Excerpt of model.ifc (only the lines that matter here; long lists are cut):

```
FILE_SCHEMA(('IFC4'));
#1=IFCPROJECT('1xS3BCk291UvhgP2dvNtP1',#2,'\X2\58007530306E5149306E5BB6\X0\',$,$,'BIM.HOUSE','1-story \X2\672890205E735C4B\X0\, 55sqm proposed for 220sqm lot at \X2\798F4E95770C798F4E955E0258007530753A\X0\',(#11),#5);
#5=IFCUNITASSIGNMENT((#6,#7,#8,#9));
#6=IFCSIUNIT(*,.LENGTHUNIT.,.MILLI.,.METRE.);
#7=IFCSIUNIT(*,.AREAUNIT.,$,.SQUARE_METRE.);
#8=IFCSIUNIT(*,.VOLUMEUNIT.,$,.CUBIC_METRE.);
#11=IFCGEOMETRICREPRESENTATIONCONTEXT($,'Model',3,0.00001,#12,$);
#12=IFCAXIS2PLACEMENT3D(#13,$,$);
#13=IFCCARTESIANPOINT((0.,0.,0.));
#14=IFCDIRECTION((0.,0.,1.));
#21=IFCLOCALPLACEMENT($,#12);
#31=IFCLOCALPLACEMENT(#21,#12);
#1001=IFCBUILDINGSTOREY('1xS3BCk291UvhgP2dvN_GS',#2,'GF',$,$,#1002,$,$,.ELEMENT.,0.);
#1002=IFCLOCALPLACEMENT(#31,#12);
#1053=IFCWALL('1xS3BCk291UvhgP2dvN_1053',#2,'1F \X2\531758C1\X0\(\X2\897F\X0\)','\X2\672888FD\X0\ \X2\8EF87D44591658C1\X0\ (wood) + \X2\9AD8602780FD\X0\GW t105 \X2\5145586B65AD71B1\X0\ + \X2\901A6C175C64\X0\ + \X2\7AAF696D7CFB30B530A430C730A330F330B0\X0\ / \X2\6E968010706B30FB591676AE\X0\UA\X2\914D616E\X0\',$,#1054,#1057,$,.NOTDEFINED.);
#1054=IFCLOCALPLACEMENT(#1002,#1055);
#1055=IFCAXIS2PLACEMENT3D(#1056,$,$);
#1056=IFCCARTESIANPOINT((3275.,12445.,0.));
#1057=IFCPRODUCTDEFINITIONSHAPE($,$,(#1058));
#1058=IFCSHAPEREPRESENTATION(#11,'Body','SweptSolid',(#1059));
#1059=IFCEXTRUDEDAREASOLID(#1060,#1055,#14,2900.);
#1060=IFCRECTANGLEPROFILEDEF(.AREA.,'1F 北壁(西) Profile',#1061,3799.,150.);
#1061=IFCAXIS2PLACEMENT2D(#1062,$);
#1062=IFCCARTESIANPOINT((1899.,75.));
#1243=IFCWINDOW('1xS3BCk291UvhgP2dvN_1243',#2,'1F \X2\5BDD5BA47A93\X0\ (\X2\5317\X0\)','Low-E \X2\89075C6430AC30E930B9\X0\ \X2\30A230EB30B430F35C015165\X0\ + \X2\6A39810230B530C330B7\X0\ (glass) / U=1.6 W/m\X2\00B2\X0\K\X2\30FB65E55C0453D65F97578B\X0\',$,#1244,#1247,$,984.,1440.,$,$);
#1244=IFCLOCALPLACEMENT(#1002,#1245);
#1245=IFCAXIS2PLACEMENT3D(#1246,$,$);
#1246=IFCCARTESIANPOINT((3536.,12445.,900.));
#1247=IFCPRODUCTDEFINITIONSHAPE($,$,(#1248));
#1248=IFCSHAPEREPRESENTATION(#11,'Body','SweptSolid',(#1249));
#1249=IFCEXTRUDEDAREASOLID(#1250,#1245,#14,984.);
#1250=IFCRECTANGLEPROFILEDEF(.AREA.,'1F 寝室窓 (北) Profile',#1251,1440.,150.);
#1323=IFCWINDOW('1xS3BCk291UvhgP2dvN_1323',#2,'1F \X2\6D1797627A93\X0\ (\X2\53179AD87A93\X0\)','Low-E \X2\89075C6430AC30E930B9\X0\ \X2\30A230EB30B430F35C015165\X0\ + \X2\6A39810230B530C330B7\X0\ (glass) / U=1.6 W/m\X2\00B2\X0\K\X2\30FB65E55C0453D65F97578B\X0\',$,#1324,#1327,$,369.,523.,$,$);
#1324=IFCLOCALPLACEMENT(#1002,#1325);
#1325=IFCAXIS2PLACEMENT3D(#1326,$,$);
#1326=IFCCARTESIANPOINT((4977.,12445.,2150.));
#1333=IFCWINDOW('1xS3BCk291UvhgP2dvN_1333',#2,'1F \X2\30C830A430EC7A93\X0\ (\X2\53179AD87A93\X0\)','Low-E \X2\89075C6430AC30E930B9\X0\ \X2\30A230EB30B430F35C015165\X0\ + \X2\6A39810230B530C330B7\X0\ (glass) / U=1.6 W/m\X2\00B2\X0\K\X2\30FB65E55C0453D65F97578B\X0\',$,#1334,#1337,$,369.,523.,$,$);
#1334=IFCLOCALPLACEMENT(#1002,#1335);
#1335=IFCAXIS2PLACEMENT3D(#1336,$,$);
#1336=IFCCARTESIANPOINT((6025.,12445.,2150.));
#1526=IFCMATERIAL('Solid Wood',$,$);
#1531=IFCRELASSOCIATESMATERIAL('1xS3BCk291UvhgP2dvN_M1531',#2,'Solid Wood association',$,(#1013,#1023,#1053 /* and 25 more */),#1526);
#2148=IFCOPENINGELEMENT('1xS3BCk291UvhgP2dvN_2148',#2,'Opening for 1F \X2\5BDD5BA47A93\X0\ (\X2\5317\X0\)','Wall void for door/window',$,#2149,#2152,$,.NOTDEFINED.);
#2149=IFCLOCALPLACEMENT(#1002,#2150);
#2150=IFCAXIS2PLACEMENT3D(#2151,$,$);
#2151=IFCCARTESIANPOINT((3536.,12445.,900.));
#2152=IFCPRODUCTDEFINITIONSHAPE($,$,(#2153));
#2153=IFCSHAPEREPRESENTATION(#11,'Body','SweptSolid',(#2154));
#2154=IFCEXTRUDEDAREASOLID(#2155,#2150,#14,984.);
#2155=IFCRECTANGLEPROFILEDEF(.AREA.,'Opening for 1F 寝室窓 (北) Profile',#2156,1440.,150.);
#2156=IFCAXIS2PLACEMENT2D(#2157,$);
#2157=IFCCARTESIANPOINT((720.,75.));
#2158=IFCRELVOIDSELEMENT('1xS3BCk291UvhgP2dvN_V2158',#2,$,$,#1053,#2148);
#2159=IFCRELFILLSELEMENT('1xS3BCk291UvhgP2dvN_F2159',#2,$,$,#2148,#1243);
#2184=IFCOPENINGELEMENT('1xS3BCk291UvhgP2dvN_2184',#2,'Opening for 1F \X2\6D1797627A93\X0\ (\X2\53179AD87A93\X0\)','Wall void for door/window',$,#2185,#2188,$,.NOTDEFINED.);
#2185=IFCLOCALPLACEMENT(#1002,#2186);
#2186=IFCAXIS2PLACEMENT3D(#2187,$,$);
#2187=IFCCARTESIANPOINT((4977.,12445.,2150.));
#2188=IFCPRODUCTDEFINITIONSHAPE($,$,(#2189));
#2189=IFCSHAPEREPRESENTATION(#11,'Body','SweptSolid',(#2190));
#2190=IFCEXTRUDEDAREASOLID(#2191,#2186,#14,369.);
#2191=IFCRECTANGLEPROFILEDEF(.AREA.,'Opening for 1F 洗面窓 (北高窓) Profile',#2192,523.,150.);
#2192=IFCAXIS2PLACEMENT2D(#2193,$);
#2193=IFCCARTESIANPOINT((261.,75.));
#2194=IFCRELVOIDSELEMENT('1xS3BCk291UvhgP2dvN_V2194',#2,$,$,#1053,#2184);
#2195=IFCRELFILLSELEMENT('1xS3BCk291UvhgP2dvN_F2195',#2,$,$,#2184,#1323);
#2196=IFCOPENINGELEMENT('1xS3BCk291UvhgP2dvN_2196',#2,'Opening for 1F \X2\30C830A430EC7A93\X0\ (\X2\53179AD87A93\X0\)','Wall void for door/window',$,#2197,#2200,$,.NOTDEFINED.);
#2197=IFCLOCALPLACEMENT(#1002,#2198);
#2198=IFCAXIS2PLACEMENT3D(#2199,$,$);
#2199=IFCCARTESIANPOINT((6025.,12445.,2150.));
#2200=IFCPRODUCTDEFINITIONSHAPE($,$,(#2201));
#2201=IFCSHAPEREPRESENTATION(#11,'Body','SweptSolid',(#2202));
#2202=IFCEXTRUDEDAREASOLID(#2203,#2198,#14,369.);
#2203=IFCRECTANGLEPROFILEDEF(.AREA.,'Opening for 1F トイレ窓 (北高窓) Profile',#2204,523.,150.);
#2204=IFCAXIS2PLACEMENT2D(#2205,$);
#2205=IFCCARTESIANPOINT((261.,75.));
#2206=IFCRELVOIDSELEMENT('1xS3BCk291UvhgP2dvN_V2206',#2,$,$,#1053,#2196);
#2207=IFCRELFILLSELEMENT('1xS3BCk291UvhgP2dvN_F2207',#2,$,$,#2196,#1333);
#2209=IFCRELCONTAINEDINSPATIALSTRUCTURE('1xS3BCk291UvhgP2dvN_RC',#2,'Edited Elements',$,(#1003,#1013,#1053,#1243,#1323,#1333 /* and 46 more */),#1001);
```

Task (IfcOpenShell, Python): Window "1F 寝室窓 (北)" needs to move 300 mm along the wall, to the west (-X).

```python
import ifcopenshell
import ifcopenshell.api.geometry
import ifcopenshell.util.placement
import ifcopenshell.util.unit

model = ifcopenshell.open("model.ifc")
unit_scale = ifcopenshell.util.unit.calculate_unit_scale(model)

window = model.by_guid("1xS3BCk291UvhgP2dvN_1243")
opening = window.FillsVoids[0].RelatingOpeningElement
wall = opening.VoidsElements[0].RelatingBuildingElement

wall_matrix = ifcopenshell.util.placement.get_local_placement(wall.ObjectPlacement)
shift = wall_matrix[:3, 0] * -0.3 / unit_scale
before = ifcopenshell.util.placement.get_local_placement(window.ObjectPlacement)[:3, 3].copy()

# The window is not placed relative to its opening, so move both.
for product in (opening, window):
    matrix = ifcopenshell.util.placement.get_local_placement(product.ObjectPlacement)
    matrix[:3, 3] += shift
    ifcopenshell.api.geometry.edit_object_placement(model, product=product, matrix=matrix, is_si=False)

after = ifcopenshell.util.placement.get_local_placement(window.ObjectPlacement)[:3, 3]
print("window moved by", (after - before).round(3) + 0.0)

model.write("model_v2.ifc")
```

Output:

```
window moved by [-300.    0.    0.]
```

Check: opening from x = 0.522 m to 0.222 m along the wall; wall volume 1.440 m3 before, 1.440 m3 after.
